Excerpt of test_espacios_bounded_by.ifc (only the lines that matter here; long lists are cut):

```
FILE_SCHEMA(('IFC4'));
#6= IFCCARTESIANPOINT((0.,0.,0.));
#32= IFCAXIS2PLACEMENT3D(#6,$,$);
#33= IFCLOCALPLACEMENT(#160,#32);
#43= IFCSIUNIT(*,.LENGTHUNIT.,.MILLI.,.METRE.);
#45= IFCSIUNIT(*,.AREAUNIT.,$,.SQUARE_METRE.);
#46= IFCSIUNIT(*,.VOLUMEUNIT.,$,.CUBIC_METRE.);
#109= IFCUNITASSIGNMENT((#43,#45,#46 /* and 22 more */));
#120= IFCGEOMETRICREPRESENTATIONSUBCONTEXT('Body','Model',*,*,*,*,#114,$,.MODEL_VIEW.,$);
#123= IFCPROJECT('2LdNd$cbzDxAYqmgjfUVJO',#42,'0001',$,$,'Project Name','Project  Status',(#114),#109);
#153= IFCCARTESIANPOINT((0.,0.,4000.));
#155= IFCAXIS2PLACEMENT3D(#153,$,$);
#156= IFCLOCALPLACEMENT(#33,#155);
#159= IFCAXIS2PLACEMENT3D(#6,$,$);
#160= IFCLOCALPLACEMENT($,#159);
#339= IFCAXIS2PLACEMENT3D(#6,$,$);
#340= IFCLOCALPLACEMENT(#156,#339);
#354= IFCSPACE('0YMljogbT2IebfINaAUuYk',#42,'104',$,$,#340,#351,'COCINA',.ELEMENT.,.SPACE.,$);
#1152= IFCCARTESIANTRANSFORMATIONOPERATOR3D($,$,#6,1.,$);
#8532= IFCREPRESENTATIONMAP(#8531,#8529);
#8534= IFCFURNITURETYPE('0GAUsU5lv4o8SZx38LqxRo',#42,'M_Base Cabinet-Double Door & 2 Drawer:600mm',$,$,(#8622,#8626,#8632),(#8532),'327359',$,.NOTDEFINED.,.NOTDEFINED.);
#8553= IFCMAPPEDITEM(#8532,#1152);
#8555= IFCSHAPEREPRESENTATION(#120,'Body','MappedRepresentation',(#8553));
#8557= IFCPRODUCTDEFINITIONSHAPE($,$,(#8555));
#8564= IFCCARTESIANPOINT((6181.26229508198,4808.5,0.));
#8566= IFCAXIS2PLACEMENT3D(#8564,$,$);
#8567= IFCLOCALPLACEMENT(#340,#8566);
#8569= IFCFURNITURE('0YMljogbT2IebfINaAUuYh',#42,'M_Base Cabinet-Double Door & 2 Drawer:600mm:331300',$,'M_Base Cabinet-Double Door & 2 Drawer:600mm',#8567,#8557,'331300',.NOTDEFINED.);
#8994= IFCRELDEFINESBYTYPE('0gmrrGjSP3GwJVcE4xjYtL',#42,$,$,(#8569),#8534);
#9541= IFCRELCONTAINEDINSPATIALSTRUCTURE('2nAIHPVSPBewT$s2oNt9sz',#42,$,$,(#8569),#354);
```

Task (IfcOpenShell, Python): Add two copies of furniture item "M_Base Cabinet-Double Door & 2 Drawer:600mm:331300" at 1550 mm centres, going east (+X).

```python
import numpy as np
import ifcopenshell
import ifcopenshell.api.geometry
import ifcopenshell.api.root
import ifcopenshell.util.element
import ifcopenshell.util.placement
import ifcopenshell.util.unit

model = ifcopenshell.open("test_espacios_bounded_by.ifc")
unit_scale = ifcopenshell.util.unit.calculate_unit_scale(model)


def reuse_history(source, copy):
    """copy_class also copies each property set's owner history, people and application; keep the originals."""
    for rel in copy.IsDefinedBy:
        if rel.is_a("IfcRelDefinesByProperties") and (history := rel.RelatingPropertyDefinition.OwnerHistory):
            rel.RelatingPropertyDefinition.OwnerHistory = source.OwnerHistory
            ifcopenshell.util.element.remove_deep2(model, history)


source = model.by_guid("0YMljogbT2IebfINaAUuYh")
base = ifcopenshell.util.placement.get_local_placement(source.ObjectPlacement)
step = np.array([1.0, 0.0, 0.0]) * 1.55 / unit_scale

for i in range(1, 3):
    copy = ifcopenshell.api.root.copy_class(model, product=source)
    copy.Representation = ifcopenshell.util.element.copy_deep(
        model, source.Representation, exclude=["IfcGeometricRepresentationContext", "IfcRepresentationMap"]
    )
    copy.Name = "M_Base Cabinet-Double Door & 2 Drawer:600mm"
    copy.Tag = None
    reuse_history(source, copy)
    matrix = base.copy()
    matrix[:3, 3] += i * step
    print("added at", matrix[:3, 3].round(3) + 0.0)
    ifcopenshell.api.geometry.edit_object_placement(model, product=copy, matrix=matrix, is_si=False)

model.write("test_espacios_bounded_by_updated.ifc")
```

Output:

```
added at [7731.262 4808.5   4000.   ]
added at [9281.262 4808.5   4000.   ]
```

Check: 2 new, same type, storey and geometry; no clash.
